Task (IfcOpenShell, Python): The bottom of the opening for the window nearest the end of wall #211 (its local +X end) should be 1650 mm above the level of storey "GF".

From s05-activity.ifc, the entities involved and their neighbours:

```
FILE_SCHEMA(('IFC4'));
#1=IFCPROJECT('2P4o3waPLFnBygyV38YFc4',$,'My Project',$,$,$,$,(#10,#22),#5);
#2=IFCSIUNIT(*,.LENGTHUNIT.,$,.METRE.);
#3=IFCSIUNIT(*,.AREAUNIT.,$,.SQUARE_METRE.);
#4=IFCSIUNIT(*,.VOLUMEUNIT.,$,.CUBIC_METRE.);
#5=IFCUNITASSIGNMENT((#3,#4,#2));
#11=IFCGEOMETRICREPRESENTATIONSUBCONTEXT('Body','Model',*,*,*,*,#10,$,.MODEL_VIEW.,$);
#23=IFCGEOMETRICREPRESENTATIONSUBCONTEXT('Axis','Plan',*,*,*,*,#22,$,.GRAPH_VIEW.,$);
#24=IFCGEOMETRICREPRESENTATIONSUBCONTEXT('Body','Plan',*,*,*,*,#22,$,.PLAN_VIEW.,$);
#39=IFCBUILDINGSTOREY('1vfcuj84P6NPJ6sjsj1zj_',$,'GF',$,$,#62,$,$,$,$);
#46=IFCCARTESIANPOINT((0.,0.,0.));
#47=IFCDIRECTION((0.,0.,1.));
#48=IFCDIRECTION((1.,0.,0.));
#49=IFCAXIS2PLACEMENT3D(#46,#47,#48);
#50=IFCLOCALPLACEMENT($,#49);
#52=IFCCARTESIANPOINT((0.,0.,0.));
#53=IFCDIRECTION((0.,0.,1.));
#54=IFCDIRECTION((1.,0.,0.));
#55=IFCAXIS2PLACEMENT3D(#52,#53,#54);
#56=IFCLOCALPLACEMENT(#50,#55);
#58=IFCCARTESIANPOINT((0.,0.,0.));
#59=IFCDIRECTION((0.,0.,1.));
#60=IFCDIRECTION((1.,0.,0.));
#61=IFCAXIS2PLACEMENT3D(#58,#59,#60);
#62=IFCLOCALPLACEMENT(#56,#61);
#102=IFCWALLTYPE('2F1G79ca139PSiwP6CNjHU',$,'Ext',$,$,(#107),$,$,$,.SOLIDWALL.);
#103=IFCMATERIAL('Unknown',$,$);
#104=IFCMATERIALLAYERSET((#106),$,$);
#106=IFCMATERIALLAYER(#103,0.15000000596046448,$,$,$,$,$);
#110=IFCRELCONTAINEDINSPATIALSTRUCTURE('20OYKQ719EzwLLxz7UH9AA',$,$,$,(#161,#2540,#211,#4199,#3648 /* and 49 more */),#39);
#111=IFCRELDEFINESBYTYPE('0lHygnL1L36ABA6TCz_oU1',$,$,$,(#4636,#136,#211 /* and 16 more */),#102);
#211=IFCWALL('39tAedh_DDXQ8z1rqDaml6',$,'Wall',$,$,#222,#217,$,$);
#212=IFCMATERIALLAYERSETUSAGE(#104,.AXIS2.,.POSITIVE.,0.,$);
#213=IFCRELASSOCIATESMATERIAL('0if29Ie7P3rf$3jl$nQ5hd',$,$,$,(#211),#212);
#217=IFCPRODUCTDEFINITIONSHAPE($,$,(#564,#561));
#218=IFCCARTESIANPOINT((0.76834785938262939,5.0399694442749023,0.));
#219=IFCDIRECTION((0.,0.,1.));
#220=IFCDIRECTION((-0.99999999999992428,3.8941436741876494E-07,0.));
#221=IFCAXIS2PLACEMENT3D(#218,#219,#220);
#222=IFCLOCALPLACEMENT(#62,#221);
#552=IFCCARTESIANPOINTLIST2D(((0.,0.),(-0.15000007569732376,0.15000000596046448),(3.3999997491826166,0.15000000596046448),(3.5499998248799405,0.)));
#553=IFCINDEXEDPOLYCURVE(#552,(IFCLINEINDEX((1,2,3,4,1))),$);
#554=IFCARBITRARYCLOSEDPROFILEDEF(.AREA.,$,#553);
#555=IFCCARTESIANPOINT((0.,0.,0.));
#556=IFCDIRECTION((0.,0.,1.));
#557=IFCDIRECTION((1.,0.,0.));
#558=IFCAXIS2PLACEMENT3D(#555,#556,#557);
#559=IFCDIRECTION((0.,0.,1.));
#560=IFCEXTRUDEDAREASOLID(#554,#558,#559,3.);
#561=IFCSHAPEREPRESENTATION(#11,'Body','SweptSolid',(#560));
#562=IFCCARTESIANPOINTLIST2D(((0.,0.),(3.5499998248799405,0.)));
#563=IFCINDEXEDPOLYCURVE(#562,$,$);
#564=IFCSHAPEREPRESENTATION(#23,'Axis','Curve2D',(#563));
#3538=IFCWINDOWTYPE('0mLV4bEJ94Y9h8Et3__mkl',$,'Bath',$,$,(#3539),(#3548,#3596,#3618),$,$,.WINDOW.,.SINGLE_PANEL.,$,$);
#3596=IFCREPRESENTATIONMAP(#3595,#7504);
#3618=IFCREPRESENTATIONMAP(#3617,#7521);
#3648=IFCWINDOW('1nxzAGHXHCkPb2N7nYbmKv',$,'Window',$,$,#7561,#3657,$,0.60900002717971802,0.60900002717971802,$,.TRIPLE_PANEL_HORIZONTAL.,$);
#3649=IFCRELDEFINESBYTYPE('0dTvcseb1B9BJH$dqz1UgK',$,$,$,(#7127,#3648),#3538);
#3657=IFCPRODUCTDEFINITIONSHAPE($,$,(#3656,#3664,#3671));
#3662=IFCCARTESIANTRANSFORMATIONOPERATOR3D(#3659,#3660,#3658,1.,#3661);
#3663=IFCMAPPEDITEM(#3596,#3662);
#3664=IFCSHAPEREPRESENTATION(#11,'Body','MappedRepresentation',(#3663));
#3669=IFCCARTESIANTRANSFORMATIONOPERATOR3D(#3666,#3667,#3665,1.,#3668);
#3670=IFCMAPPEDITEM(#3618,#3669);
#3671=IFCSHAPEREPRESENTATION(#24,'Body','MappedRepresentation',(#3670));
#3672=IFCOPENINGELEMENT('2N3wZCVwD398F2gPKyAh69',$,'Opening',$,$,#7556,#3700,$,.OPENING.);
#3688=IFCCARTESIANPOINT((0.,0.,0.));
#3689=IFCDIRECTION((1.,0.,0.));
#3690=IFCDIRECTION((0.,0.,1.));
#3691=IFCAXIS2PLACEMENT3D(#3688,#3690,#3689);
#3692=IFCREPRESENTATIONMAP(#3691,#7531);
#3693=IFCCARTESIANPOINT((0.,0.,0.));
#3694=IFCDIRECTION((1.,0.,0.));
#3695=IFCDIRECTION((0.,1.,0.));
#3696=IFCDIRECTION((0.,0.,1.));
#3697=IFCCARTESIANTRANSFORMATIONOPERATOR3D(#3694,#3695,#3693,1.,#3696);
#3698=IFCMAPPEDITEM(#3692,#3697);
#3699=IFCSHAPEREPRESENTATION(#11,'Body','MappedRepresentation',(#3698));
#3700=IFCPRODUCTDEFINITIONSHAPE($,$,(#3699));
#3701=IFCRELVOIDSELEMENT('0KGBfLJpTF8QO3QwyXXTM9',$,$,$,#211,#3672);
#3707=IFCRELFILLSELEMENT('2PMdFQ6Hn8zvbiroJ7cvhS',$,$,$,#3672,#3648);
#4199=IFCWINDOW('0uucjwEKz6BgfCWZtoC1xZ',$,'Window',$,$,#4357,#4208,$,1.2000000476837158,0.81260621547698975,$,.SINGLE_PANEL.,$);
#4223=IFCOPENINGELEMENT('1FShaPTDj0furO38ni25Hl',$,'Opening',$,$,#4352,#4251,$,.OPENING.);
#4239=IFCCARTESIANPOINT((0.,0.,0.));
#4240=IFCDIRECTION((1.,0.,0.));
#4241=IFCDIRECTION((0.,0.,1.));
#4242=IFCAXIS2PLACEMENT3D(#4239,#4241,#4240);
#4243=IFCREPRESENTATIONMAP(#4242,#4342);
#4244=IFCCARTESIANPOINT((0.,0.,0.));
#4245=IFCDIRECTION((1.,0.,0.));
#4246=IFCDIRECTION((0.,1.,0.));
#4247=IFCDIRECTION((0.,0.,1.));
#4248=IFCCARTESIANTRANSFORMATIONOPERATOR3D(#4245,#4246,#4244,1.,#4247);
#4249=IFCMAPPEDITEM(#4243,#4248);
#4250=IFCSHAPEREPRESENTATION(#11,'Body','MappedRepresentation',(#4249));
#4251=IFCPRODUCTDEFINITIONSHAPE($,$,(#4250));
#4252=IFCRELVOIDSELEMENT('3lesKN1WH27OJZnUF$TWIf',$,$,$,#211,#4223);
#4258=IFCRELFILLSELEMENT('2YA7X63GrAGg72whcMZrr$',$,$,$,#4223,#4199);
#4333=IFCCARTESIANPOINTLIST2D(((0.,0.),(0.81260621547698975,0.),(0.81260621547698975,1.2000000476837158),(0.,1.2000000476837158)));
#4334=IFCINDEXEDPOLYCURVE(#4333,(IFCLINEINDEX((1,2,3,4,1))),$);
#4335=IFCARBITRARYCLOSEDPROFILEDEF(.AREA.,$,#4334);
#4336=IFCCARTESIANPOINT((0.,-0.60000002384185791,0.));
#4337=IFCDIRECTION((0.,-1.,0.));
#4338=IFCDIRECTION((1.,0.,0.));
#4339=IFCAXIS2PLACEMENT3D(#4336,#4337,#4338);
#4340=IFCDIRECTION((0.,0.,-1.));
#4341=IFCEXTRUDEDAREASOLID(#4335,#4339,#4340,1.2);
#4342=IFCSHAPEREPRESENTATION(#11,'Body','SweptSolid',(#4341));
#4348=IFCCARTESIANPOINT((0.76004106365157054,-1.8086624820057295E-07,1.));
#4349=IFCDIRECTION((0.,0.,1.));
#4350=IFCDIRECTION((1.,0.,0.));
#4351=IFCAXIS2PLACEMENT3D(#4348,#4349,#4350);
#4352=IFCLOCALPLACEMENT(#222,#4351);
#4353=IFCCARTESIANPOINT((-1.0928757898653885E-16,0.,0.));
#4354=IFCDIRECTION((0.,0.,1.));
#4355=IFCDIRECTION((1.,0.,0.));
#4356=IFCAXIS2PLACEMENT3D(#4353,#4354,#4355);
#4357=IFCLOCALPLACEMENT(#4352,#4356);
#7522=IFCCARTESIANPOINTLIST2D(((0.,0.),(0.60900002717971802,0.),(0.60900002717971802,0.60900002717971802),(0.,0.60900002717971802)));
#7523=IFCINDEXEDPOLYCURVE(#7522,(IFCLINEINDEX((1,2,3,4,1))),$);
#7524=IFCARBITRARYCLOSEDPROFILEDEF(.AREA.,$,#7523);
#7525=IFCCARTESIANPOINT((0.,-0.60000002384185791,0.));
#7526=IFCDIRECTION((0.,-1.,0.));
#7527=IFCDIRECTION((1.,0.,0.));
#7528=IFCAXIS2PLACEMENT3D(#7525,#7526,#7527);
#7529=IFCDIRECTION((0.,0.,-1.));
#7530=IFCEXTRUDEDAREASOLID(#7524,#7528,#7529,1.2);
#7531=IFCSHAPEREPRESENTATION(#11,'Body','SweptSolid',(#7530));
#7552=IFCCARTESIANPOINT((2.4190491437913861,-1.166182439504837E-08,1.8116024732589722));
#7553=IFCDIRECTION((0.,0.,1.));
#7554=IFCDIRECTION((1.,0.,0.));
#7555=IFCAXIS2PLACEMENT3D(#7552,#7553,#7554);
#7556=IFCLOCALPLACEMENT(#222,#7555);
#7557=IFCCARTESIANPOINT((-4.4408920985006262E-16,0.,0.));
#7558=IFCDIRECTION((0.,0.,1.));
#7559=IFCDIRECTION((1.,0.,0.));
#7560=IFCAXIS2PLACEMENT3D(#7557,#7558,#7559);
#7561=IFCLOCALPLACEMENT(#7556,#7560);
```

```python
import numpy as np
import ifcopenshell
import ifcopenshell.api.geometry
import ifcopenshell.geom
import ifcopenshell.util.element
import ifcopenshell.util.placement
import ifcopenshell.util.shape
import ifcopenshell.util.unit

model = ifcopenshell.open("s05-activity.ifc")
unit_scale = ifcopenshell.util.unit.calculate_unit_scale(model)

window = model.by_guid("1nxzAGHXHCkPb2N7nYbmKv")
opening = window.FillsVoids[0].RelatingOpeningElement
storey = ifcopenshell.util.element.get_container(window, ifc_class="IfcBuildingStorey")
level = ifcopenshell.util.placement.get_local_placement(storey.ObjectPlacement)[2, 3]

# The opening's origin need not be at the sill, so measure its lowest point.
shape = ifcopenshell.geom.create_shape(ifcopenshell.geom.settings(), opening)
bottom = ifcopenshell.util.shape.get_shape_bottom_elevation(shape, shape.geometry) / unit_scale
dz = level + 1.65 - bottom

shift = np.array([0.0, 0.0, dz])
# The window is placed relative to its opening, so it follows when the opening moves.
matrix = ifcopenshell.util.placement.get_local_placement(opening.ObjectPlacement)
matrix[:3, 3] += shift
ifcopenshell.api.geometry.edit_object_placement(
    model, product=opening, matrix=matrix, is_si=False, should_transform_children=True
)

print(f"moved by {dz * unit_scale:+.3f} m")

model.write("s05-activity_updated.ifc")
```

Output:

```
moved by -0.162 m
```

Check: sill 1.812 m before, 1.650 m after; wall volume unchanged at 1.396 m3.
